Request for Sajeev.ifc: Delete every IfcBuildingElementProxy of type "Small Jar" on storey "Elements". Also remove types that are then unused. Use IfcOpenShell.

First a look at what the model holds.

```python
import ifcopenshell
import ifcopenshell.util.element

model = ifcopenshell.open("Sajeev.ifc")
print(model.schema)
storey = next(s for s in model.by_type("IfcBuildingStorey") if s.Name == "Elements")
proxies = [e for e in ifcopenshell.util.element.get_decomposition(storey) if e.is_a("IfcBuildingElementProxy")]
seen = {}
for e in proxies:
    element_type = ifcopenshell.util.element.get_type(e)
    name = element_type.Name if element_type not in (None, e) else None
    seen[name] = seen.get(name, 0) + 1
for name, count in sorted(seen.items(), key=str):
    print(count, "x", name)
```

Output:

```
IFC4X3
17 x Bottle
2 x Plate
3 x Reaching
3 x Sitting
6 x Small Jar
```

```python
import ifcopenshell
import ifcopenshell.api.root
import ifcopenshell.util.element

model = ifcopenshell.open("Sajeev.ifc")

storey = next(s for s in model.by_type("IfcBuildingStorey") if s.Name == "Elements")
proxies = [e for e in ifcopenshell.util.element.get_decomposition(storey) if e.is_a("IfcBuildingElementProxy")]
targets = [e for e in proxies if (t := ifcopenshell.util.element.get_type(e)) not in (None, e) and t.Name == "Small Jar"]
types = {ifcopenshell.util.element.get_type(e) for e in targets} - {None, *targets}

for e in targets:
    ifcopenshell.api.root.remove_product(model, product=e)
print(len(targets), "removed")

unused = [t for t in types if not ifcopenshell.util.element.get_types(t)]
for t in unused:
    ifcopenshell.api.root.remove_product(model, product=t)
print(len(unused), "unused types removed")

model.write("Sajeev_v2.ifc")
```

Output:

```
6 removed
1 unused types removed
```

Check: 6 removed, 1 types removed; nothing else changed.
